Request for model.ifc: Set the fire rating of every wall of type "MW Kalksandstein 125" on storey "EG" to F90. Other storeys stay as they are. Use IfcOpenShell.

First a look at what the model holds.

```python
import ifcopenshell
import ifcopenshell.util.element

model = ifcopenshell.open("model.ifc")
print(model.schema)
storey = next(s for s in model.by_type("IfcBuildingStorey") if s.Name == "EG")
walls = [e for e in ifcopenshell.util.element.get_decomposition(storey) if e.is_a("IfcWall")]
seen = {}
for e in walls:
    element_type = ifcopenshell.util.element.get_type(e)
    key = (element_type.Name if element_type != e and element_type else None, ifcopenshell.util.element.get_pset(e, "Pset_WallCommon", "FireRating"))
    seen[key] = seen.get(key, 0) + 1
for (name, value), count in sorted(seen.items(), key=str):
    print(count, "x", name, "|", value)
```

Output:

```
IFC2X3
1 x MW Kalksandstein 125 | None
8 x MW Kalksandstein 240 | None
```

```python
import ifcopenshell
import ifcopenshell.api.pset
import ifcopenshell.util.element

model = ifcopenshell.open("model.ifc")

storey = next(s for s in model.by_type("IfcBuildingStorey") if s.Name == "EG")
walls = [e for e in ifcopenshell.util.element.get_decomposition(storey) if e.is_a("IfcWall")]

count = 0
for e in walls:
    element_type = ifcopenshell.util.element.get_type(e)
    if element_type in (None, e) or element_type.Name != "MW Kalksandstein 125":
        continue
    # add_pset returns the element's existing set when there is one.
    pset = ifcopenshell.api.pset.add_pset(model, product=e, name="Pset_WallCommon")
    ifcopenshell.api.pset.edit_pset(model, pset=pset, properties={"FireRating": "F90"})
    count += 1

print(count, "walls updated")

model.write("model-out.ifc")
```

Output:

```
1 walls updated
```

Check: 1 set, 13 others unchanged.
